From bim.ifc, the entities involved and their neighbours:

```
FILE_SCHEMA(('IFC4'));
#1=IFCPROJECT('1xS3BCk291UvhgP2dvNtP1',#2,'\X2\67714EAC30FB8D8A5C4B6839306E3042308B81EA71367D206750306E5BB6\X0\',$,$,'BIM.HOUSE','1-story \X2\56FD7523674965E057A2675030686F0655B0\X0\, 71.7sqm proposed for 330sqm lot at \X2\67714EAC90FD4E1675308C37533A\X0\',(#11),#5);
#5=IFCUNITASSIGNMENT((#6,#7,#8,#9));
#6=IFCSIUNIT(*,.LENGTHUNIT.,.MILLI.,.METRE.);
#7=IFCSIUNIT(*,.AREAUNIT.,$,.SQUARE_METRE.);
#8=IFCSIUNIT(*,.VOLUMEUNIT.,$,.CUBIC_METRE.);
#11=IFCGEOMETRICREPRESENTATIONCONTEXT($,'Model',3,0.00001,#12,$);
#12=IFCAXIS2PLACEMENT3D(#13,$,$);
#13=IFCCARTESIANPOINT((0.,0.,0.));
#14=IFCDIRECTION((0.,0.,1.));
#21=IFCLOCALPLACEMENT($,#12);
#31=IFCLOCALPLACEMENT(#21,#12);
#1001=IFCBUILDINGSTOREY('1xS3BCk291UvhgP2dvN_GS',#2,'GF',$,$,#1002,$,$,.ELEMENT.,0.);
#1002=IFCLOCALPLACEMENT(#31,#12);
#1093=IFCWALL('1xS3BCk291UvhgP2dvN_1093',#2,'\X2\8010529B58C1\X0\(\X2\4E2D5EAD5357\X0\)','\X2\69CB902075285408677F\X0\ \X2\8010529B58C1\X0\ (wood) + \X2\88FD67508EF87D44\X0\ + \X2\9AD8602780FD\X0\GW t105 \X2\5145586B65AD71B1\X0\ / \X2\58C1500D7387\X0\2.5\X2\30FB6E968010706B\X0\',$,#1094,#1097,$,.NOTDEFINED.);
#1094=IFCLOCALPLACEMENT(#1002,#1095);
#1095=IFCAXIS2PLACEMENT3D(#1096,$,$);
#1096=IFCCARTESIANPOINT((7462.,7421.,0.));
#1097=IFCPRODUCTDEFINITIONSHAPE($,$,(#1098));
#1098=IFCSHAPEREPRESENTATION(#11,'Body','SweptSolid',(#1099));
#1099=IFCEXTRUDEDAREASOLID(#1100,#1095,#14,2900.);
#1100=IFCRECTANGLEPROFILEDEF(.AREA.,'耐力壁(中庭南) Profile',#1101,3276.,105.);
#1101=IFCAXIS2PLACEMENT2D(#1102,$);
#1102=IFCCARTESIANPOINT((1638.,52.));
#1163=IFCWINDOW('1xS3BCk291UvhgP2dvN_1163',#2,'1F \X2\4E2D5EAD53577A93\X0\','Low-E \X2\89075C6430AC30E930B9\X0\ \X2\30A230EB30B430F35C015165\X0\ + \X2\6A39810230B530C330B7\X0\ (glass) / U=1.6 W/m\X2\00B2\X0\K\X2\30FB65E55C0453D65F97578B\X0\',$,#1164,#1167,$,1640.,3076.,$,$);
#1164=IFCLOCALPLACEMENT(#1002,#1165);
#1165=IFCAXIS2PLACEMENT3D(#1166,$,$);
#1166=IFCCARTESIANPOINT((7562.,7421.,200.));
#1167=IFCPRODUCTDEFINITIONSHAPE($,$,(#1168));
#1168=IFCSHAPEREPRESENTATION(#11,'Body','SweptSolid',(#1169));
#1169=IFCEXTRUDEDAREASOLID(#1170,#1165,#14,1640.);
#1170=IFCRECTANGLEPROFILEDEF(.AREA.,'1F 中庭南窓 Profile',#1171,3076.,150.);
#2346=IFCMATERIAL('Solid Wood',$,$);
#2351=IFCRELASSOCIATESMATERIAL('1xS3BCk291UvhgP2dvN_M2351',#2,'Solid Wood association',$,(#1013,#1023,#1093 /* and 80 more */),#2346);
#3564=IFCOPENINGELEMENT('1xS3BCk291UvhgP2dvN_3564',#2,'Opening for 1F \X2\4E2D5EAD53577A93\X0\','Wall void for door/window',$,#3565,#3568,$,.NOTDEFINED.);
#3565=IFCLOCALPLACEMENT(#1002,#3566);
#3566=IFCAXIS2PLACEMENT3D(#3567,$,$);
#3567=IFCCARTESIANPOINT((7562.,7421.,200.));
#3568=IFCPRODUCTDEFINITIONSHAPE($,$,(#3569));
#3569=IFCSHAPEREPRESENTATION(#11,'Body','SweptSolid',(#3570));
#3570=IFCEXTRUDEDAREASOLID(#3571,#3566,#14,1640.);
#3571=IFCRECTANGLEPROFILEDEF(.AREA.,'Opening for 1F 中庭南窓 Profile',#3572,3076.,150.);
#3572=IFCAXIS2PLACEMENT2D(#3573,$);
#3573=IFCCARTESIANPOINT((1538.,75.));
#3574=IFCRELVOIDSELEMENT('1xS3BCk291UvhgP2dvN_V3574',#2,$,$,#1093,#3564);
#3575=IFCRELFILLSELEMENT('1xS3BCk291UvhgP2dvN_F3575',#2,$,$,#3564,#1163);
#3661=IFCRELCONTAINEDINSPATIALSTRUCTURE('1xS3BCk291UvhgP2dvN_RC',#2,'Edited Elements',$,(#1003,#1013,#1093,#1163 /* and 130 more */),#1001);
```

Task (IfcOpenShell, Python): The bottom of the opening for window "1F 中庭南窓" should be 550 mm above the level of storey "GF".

```python
import numpy as np
import ifcopenshell
import ifcopenshell.api.geometry
import ifcopenshell.geom
import ifcopenshell.util.element
import ifcopenshell.util.placement
import ifcopenshell.util.shape
import ifcopenshell.util.unit

model = ifcopenshell.open("bim.ifc")
unit_scale = ifcopenshell.util.unit.calculate_unit_scale(model)

window = model.by_guid("1xS3BCk291UvhgP2dvN_1163")
opening = window.FillsVoids[0].RelatingOpeningElement
storey = ifcopenshell.util.element.get_container(window, ifc_class="IfcBuildingStorey")
level = ifcopenshell.util.placement.get_local_placement(storey.ObjectPlacement)[2, 3]

# The opening's origin need not be at the sill, so measure its lowest point.
shape = ifcopenshell.geom.create_shape(ifcopenshell.geom.settings(), opening)
bottom = ifcopenshell.util.shape.get_shape_bottom_elevation(shape, shape.geometry) / unit_scale
dz = level + 550.0 - bottom

shift = np.array([0.0, 0.0, dz])
# The window is not placed relative to its opening, so move both.
for product in (opening, window):
    matrix = ifcopenshell.util.placement.get_local_placement(product.ObjectPlacement)
    matrix[:3, 3] += shift
    ifcopenshell.api.geometry.edit_object_placement(model, product=product, matrix=matrix, is_si=False)

print(f"moved by {dz * unit_scale:+.3f} m")

model.write("bim_edited.ifc")
```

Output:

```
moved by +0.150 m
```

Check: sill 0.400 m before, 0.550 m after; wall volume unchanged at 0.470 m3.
